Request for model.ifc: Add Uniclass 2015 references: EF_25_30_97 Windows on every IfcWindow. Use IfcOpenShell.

First a look at what the model holds.

```python
import ifcopenshell

model = ifcopenshell.open("model.ifc")
print(model.schema)
print("classifications:", [c.Name for c in model.by_type("IfcClassification")])
for ifc_class in ("IfcDoor", "IfcRoof", "IfcStair", "IfcWall", "IfcWindow"):
    print(ifc_class, len(model.by_type(ifc_class)))
```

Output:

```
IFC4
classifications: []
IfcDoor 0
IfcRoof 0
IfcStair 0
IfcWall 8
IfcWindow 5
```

```python
import ifcopenshell
import ifcopenshell.api.classification

model = ifcopenshell.open("model.ifc")

system = ifcopenshell.api.classification.add_classification(model, classification="Uniclass 2015")

codes = {
    "IfcWindow": ("EF_25_30_97", "Windows"),
}
for ifc_class, (code, name) in codes.items():
    products = model.by_type(ifc_class)
    ifcopenshell.api.classification.add_reference(
        model, products=products, classification=system, identification=code, name=name
    )
    print(code, len(products))

model.write("model_v2.ifc")
```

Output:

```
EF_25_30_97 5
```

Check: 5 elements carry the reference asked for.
